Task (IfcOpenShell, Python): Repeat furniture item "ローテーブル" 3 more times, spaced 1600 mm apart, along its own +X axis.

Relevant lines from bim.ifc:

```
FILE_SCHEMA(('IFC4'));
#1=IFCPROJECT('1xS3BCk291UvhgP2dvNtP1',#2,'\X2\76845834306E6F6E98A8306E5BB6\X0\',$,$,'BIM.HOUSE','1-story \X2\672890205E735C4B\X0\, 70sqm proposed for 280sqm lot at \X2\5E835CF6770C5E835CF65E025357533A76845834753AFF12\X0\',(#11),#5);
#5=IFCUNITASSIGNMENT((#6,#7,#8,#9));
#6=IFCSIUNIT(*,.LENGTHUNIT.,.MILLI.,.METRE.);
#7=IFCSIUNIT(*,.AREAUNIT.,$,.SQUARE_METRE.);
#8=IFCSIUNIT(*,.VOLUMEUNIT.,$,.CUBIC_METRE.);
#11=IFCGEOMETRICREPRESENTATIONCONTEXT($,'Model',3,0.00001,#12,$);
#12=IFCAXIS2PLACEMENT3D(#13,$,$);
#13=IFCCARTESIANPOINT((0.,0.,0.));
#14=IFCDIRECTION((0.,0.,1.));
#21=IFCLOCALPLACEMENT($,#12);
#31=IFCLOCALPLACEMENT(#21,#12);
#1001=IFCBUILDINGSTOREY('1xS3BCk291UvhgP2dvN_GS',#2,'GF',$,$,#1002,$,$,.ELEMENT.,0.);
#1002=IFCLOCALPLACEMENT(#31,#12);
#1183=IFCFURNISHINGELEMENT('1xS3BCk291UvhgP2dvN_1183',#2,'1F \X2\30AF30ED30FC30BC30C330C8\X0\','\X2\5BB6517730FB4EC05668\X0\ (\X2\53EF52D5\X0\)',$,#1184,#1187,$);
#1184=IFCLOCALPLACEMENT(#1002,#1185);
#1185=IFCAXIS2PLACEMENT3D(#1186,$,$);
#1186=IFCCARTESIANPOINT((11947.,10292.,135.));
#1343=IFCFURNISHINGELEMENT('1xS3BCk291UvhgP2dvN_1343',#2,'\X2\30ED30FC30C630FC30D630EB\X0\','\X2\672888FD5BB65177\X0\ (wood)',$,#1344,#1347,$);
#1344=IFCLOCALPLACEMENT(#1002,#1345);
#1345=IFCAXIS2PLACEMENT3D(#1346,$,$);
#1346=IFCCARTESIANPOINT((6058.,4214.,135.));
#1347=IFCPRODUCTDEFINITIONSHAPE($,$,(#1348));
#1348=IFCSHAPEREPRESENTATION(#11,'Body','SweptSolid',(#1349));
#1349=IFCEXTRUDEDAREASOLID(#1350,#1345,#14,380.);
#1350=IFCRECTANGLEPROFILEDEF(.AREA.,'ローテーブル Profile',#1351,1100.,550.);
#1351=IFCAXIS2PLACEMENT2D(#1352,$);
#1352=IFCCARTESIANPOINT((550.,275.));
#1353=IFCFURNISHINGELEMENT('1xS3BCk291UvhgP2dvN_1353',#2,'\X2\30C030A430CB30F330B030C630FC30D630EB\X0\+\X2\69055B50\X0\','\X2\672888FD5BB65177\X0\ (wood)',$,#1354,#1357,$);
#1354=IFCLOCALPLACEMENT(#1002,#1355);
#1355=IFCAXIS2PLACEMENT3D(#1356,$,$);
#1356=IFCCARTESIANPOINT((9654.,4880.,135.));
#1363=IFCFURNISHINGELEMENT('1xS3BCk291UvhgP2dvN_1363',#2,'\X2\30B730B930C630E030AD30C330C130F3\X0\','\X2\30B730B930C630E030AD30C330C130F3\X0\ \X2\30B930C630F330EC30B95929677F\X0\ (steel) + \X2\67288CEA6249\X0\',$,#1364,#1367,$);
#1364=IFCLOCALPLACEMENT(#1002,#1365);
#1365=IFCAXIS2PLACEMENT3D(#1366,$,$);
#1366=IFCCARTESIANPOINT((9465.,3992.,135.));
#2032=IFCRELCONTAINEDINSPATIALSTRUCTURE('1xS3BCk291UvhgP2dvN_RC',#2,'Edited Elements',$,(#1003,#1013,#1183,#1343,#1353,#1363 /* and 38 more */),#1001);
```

```python
import ifcopenshell
import ifcopenshell.api.geometry
import ifcopenshell.api.root
import ifcopenshell.util.element
import ifcopenshell.util.placement

model = ifcopenshell.open("bim.ifc")


def reuse_history(source, copy):
    """copy_class also copies each property set's owner history, people and application; keep the originals."""
    for rel in copy.IsDefinedBy:
        if rel.is_a("IfcRelDefinesByProperties") and (history := rel.RelatingPropertyDefinition.OwnerHistory):
            rel.RelatingPropertyDefinition.OwnerHistory = source.OwnerHistory
            ifcopenshell.util.element.remove_deep2(model, history)


source = model.by_guid("1xS3BCk291UvhgP2dvN_1343")
base = ifcopenshell.util.placement.get_local_placement(source.ObjectPlacement)
step = base[:3, 0] * 1600.0

for i in range(1, 4):
    copy = ifcopenshell.api.root.copy_class(model, product=source)
    copy.Representation = ifcopenshell.util.element.copy_deep(
        model, source.Representation, exclude=["IfcGeometricRepresentationContext", "IfcRepresentationMap"]
    )
    reuse_history(source, copy)
    matrix = base.copy()
    matrix[:3, 3] += i * step
    print("added at", matrix[:3, 3].round(3) + 0.0)
    ifcopenshell.api.geometry.edit_object_placement(model, product=copy, matrix=matrix, is_si=False)

model.write("bim_v2.ifc")
```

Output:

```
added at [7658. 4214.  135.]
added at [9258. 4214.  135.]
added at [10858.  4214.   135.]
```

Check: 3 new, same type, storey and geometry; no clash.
